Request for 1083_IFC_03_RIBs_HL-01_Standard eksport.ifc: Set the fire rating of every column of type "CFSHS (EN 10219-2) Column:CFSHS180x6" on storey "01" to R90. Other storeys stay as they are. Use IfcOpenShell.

First a look at what the model holds.

```python
import ifcopenshell
import ifcopenshell.util.element

model = ifcopenshell.open("1083_IFC_03_RIBs_HL-01_Standard eksport.ifc")
print(model.schema)
storey = next(s for s in model.by_type("IfcBuildingStorey") if s.Name == "01")
columns = [e for e in ifcopenshell.util.element.get_decomposition(storey) if e.is_a("IfcColumn")]
seen = {}
for e in columns:
    element_type = ifcopenshell.util.element.get_type(e)
    key = (element_type.Name if element_type != e and element_type else None, ifcopenshell.util.element.get_pset(e, "Pset_ColumnCommon", "FireRating"))
    seen[key] = seen.get(key, 0) + 1
for (name, value), count in sorted(seen.items(), key=str):
    print(count, "x", name, "|", value)
```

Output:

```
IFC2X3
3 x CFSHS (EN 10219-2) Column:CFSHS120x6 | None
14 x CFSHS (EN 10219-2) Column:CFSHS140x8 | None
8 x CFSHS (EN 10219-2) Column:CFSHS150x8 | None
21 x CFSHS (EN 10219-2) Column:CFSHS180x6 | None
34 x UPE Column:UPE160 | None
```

```python
import ifcopenshell
import ifcopenshell.api.pset
import ifcopenshell.util.element

model = ifcopenshell.open("1083_IFC_03_RIBs_HL-01_Standard eksport.ifc")

storey = next(s for s in model.by_type("IfcBuildingStorey") if s.Name == "01")
columns = [e for e in ifcopenshell.util.element.get_decomposition(storey) if e.is_a("IfcColumn")]

count = 0
for e in columns:
    element_type = ifcopenshell.util.element.get_type(e)
    if element_type in (None, e) or element_type.Name != "CFSHS (EN 10219-2) Column:CFSHS180x6":
        continue
    # add_pset returns the element's existing set when there is one.
    pset = ifcopenshell.api.pset.add_pset(model, product=e, name="Pset_ColumnCommon")
    ifcopenshell.api.pset.edit_pset(model, pset=pset, properties={"FireRating": "R90"})
    count += 1

print(count, "columns updated")

model.write("1083_IFC_03_RIBs_HL-01_Standard eksport-out.ifc")
```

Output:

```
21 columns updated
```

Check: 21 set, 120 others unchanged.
